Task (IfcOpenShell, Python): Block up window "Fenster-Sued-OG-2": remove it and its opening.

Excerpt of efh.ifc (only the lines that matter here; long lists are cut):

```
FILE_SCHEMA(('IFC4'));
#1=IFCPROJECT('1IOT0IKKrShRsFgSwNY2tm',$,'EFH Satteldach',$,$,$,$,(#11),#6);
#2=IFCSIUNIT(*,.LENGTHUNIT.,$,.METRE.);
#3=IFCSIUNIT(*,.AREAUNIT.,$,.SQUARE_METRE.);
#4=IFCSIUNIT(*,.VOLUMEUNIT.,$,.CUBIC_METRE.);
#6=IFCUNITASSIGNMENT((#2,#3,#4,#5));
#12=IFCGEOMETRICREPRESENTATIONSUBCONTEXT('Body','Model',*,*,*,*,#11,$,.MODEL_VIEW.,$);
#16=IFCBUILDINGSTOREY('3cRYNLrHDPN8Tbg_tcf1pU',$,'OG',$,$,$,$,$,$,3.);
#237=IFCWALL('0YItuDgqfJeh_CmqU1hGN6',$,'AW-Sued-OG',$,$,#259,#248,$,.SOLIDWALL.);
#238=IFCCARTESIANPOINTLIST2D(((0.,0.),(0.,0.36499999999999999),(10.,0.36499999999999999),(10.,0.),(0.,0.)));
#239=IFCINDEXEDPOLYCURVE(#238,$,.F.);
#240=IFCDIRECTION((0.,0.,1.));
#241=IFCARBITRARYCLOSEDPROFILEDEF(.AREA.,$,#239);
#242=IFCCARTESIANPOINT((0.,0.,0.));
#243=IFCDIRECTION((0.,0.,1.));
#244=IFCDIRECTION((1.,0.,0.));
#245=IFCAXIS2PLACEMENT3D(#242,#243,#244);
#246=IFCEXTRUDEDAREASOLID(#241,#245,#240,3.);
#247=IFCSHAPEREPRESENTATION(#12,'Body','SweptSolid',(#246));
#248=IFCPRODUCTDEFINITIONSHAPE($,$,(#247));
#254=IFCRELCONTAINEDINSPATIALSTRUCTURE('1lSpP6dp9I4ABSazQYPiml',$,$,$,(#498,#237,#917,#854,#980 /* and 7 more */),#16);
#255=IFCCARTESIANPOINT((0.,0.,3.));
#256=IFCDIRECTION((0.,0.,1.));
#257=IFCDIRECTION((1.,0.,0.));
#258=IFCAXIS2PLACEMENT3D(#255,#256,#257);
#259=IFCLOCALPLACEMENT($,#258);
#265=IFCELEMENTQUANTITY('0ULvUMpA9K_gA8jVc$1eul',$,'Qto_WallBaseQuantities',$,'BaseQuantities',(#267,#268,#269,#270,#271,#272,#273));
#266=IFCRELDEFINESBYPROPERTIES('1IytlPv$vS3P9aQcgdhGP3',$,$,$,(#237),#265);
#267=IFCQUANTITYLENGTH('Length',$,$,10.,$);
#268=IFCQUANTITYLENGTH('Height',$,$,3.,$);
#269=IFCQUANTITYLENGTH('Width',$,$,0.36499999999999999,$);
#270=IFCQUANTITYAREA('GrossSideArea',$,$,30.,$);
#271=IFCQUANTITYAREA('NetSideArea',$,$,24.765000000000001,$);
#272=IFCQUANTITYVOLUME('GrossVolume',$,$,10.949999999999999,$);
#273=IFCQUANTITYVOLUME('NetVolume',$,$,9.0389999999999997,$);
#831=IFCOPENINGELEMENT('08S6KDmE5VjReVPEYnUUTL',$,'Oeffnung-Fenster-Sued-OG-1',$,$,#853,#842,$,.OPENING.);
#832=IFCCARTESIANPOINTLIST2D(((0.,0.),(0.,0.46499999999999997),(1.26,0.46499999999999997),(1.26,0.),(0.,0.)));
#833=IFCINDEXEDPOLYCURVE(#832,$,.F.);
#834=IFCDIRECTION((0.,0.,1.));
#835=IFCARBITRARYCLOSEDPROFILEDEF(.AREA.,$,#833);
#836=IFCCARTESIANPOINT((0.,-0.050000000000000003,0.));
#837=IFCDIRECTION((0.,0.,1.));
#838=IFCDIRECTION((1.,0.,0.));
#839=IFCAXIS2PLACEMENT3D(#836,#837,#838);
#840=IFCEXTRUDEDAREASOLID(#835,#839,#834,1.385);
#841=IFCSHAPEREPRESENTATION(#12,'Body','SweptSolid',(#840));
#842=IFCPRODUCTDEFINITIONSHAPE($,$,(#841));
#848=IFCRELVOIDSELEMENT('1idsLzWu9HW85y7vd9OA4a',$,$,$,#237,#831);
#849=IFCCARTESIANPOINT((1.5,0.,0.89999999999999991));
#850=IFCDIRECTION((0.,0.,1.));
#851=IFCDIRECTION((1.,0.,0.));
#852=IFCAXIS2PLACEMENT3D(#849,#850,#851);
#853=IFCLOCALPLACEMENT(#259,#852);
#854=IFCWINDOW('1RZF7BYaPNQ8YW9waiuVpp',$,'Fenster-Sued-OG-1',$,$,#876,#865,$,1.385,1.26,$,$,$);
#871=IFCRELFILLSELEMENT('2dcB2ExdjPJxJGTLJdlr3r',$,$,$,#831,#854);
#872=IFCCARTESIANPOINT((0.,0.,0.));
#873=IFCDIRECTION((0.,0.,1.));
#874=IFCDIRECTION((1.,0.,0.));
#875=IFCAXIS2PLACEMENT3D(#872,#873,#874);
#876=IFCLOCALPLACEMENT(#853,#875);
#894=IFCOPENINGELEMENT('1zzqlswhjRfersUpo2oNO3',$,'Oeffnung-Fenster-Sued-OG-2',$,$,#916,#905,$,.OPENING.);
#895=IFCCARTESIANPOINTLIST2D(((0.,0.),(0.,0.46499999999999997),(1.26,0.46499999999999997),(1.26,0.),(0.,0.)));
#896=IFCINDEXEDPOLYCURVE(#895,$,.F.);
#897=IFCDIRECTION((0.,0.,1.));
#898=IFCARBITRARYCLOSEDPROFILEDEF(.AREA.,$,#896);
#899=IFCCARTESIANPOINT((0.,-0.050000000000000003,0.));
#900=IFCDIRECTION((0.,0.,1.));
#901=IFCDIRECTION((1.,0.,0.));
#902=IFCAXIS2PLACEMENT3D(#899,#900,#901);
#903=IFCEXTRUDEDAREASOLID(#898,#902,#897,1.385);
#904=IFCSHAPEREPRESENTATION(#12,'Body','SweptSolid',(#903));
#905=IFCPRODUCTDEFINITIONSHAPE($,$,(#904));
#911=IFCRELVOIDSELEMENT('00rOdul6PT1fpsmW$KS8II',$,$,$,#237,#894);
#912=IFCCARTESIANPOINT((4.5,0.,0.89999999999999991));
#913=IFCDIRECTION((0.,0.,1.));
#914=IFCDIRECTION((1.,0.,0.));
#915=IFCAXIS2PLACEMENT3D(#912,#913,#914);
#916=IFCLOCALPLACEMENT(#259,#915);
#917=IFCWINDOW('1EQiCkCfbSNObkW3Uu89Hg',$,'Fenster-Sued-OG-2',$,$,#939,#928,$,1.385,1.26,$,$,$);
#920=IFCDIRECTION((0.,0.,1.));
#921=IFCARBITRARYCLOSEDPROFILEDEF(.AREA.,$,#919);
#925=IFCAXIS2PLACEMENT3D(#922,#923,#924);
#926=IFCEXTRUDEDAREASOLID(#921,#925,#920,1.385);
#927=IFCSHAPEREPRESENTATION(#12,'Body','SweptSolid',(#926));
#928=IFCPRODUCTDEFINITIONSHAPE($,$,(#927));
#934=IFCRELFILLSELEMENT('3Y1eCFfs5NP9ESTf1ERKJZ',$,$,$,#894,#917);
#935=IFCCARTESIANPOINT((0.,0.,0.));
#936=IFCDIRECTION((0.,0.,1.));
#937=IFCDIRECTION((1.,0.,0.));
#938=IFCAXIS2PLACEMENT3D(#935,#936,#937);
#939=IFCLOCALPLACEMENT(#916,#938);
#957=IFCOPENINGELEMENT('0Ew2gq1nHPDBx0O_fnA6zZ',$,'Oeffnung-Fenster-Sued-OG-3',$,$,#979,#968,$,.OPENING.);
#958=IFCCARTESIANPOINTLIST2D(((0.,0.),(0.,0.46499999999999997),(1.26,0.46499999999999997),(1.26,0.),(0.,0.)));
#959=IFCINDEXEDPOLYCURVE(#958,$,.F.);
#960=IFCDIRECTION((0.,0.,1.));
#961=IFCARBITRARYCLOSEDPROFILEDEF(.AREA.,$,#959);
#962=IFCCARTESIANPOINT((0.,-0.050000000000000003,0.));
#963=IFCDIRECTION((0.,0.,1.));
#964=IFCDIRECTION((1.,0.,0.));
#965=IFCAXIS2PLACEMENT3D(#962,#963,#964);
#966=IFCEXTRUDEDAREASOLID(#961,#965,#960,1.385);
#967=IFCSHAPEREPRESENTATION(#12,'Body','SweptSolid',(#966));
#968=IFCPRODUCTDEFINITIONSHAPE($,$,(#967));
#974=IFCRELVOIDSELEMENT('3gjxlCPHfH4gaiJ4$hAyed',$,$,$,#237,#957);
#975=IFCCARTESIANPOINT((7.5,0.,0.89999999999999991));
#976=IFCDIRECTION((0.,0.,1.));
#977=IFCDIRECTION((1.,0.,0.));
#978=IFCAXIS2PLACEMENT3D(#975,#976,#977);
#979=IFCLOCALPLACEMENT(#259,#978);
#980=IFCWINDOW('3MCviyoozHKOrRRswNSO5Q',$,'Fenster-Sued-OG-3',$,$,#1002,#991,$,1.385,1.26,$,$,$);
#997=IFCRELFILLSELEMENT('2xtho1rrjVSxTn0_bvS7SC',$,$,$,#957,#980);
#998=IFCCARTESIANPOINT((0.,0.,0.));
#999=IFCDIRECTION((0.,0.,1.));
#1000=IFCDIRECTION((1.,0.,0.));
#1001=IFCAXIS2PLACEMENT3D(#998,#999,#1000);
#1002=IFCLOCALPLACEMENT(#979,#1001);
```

```python
import ifcopenshell
import ifcopenshell.api.feature
import ifcopenshell.api.pset
import ifcopenshell.api.root
import ifcopenshell.geom
import ifcopenshell.util.element
import ifcopenshell.util.shape
import ifcopenshell.util.unit

model = ifcopenshell.open("efh.ifc")
area_scale = ifcopenshell.util.unit.calculate_unit_scale(model, "AREAUNIT")
volume_scale = ifcopenshell.util.unit.calculate_unit_scale(model, "VOLUMEUNIT")
settings = ifcopenshell.geom.settings()


def volume(element):
    """Net volume in cubic metres, openings subtracted."""
    shape = ifcopenshell.geom.create_shape(settings, element)
    return ifcopenshell.util.shape.get_volume(shape.geometry)


window = model.by_guid("1EQiCkCfbSNObkW3Uu89Hg")
opening = window.FillsVoids[0].RelatingOpeningElement
wall = opening.VoidsElements[0].RelatingBuildingElement
before = volume(wall)

ifcopenshell.api.root.remove_product(model, product=window)
ifcopenshell.api.feature.remove_feature(model, feature=opening)

after = volume(wall)
thickness = 0.365  # wall thickness in metres

# Update the wall's stored quantities.
qto = model.by_id(ifcopenshell.util.element.get_pset(wall, "Qto_WallBaseQuantities", should_inherit=False)["id"])
ifcopenshell.api.pset.edit_qto(model, qto=qto, properties={
    "NetSideArea": after / thickness / area_scale,
    "NetVolume": after / volume_scale,
})

print(f"wall volume {before:.3f} -> {after:.3f} m3")

model.write("efh_edited.ifc")
```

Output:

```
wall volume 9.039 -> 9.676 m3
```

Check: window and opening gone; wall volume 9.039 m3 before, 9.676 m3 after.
